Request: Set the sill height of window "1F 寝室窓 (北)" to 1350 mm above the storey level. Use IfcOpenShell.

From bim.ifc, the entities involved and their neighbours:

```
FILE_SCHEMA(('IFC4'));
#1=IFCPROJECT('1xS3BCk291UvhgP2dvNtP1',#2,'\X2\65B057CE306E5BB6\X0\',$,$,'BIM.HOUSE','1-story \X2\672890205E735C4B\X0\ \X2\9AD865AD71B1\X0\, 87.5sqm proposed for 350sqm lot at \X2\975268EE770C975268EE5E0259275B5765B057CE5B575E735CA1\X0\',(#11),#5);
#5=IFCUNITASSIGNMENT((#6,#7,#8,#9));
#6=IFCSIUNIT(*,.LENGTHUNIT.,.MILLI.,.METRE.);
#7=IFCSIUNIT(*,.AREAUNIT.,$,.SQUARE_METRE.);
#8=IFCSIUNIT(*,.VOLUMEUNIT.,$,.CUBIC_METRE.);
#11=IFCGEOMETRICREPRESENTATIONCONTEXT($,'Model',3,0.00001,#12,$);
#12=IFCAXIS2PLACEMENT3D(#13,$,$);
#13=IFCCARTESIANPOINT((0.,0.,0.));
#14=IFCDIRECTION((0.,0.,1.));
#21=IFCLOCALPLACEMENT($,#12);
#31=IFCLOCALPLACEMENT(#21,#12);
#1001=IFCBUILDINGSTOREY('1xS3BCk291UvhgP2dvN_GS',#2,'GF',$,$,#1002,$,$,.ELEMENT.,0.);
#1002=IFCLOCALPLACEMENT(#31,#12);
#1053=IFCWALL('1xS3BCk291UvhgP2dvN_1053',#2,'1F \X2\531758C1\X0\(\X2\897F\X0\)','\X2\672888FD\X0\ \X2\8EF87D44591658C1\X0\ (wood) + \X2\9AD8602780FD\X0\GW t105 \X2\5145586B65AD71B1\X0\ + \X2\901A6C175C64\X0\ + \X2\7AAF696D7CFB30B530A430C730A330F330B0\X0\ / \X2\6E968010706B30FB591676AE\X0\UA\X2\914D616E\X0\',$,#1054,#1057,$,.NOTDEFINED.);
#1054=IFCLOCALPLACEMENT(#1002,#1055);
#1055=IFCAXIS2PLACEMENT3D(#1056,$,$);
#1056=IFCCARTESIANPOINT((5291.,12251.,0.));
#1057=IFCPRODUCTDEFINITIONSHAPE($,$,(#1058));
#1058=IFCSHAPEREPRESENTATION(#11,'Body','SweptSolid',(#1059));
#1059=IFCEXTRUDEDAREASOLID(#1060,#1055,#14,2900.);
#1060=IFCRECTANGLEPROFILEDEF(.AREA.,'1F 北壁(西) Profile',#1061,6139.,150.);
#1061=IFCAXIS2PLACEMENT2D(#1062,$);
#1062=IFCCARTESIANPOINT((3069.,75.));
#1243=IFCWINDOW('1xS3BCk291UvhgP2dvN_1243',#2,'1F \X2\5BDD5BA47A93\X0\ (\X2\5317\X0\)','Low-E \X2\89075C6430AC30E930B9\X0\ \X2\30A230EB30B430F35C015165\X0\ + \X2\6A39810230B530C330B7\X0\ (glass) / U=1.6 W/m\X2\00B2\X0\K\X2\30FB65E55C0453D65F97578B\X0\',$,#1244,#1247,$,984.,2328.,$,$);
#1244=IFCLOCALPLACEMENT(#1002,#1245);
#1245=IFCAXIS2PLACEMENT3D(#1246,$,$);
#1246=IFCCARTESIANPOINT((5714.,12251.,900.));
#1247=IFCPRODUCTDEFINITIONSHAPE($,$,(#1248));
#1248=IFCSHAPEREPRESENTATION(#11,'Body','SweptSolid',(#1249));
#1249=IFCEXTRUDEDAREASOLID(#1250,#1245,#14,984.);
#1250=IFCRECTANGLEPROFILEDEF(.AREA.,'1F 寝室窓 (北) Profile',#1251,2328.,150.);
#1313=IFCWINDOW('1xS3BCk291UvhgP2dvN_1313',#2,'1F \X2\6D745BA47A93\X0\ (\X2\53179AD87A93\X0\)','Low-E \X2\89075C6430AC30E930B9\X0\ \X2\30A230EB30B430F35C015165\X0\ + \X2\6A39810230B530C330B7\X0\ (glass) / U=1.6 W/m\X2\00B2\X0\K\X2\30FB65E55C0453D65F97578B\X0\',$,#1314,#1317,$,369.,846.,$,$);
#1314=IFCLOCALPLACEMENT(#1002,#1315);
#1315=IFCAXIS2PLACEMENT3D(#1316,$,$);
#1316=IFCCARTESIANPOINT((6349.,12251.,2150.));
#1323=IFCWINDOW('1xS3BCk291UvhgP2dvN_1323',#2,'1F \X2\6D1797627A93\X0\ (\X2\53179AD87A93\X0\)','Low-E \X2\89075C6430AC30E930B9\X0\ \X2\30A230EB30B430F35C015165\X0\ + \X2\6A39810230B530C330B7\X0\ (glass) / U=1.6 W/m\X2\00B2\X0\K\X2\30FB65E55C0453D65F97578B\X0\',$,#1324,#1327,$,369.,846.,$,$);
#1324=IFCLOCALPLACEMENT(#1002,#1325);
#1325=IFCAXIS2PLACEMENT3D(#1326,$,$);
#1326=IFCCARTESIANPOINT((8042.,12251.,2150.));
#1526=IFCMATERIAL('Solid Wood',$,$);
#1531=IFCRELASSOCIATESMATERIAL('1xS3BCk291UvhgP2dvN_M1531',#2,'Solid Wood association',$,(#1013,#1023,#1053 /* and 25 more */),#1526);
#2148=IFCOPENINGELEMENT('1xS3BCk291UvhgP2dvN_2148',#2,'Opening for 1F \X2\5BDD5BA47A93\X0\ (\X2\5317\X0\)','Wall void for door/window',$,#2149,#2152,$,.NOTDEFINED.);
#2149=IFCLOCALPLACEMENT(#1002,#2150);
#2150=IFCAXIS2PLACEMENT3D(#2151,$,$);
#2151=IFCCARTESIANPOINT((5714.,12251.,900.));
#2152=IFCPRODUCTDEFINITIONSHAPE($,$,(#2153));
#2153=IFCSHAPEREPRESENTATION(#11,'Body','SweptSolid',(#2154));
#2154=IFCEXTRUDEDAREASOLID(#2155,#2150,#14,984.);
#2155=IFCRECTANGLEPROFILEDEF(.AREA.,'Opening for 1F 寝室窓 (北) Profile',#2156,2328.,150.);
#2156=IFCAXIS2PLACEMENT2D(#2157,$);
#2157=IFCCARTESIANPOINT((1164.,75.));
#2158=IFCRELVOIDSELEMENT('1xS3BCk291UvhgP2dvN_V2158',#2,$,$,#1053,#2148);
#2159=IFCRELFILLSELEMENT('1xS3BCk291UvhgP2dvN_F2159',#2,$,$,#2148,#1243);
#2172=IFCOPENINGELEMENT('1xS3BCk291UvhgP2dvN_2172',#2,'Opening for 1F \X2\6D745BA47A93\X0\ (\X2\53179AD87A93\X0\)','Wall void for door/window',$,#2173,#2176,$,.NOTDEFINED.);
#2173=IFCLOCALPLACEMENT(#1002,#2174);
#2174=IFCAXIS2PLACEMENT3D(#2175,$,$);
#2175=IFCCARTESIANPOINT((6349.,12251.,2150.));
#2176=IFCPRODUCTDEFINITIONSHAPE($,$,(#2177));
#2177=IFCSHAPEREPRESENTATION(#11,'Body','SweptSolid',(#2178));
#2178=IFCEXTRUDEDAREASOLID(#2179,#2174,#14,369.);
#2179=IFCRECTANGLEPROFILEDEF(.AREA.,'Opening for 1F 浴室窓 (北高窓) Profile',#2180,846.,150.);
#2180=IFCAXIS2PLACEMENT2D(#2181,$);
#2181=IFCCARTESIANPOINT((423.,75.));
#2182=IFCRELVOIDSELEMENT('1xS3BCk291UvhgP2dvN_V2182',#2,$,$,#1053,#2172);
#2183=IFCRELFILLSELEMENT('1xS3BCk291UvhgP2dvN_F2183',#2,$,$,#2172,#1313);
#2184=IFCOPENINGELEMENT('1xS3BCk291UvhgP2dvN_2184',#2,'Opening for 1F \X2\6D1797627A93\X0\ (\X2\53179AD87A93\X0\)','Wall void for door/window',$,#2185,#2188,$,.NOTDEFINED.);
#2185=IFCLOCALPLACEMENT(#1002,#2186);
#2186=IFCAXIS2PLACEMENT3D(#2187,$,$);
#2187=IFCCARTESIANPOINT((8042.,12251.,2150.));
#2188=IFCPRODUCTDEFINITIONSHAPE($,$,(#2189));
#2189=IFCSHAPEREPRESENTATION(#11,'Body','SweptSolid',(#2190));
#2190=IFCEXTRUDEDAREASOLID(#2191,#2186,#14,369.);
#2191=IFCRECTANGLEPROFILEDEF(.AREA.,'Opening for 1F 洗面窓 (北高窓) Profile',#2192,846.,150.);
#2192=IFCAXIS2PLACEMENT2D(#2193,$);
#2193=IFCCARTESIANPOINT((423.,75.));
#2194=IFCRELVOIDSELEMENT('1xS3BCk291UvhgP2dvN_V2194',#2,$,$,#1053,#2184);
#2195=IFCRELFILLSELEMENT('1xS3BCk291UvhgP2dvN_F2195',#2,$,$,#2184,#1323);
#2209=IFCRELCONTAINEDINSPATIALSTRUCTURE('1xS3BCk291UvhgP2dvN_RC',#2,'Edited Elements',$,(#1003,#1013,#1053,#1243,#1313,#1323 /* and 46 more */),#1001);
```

```python
import numpy as np
import ifcopenshell
import ifcopenshell.api.geometry
import ifcopenshell.geom
import ifcopenshell.util.element
import ifcopenshell.util.placement
import ifcopenshell.util.shape
import ifcopenshell.util.unit

model = ifcopenshell.open("bim.ifc")
unit_scale = ifcopenshell.util.unit.calculate_unit_scale(model)

window = model.by_guid("1xS3BCk291UvhgP2dvN_1243")
opening = window.FillsVoids[0].RelatingOpeningElement
storey = ifcopenshell.util.element.get_container(window, ifc_class="IfcBuildingStorey")
level = ifcopenshell.util.placement.get_local_placement(storey.ObjectPlacement)[2, 3]

# The opening's origin need not be at the sill, so measure its lowest point.
shape = ifcopenshell.geom.create_shape(ifcopenshell.geom.settings(), opening)
bottom = ifcopenshell.util.shape.get_shape_bottom_elevation(shape, shape.geometry) / unit_scale
dz = level + 1350.0 - bottom

shift = np.array([0.0, 0.0, dz])
# The window is not placed relative to its opening, so move both.
for product in (opening, window):
    matrix = ifcopenshell.util.placement.get_local_placement(product.ObjectPlacement)
    matrix[:3, 3] += shift
    ifcopenshell.api.geometry.edit_object_placement(model, product=product, matrix=matrix, is_si=False)

print(f"moved by {dz * unit_scale:+.3f} m")

model.write("bim_edited.ifc")
```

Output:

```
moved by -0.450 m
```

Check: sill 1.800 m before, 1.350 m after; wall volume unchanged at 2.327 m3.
